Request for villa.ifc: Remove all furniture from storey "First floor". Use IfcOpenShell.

First a look at what the model holds.

```python
import ifcopenshell
import ifcopenshell.util.element

model = ifcopenshell.open("villa.ifc")
print(model.schema)
storey = next(s for s in model.by_type("IfcBuildingStorey") if s.Name == "First floor")
furniture = [e for e in ifcopenshell.util.element.get_decomposition(storey) if e.is_a("IfcFurnishingElement")]
seen = {}
for e in furniture:
    element_type = ifcopenshell.util.element.get_type(e)
    name = element_type.Name if element_type not in (None, e) else None
    seen[name] = seen.get(name, 0) + 1
for name, count in sorted(seen.items(), key=str):
    print(count, "x", name)
```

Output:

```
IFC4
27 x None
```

```python
import ifcopenshell
import ifcopenshell.api.root
import ifcopenshell.util.element

model = ifcopenshell.open("villa.ifc")

storey = next(s for s in model.by_type("IfcBuildingStorey") if s.Name == "First floor")
furniture = [e for e in ifcopenshell.util.element.get_decomposition(storey) if e.is_a("IfcFurnishingElement")]

for e in furniture:
    ifcopenshell.api.root.remove_product(model, product=e)
print(len(furniture), "removed")

model.write("villa_rev.ifc")
```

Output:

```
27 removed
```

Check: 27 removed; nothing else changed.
